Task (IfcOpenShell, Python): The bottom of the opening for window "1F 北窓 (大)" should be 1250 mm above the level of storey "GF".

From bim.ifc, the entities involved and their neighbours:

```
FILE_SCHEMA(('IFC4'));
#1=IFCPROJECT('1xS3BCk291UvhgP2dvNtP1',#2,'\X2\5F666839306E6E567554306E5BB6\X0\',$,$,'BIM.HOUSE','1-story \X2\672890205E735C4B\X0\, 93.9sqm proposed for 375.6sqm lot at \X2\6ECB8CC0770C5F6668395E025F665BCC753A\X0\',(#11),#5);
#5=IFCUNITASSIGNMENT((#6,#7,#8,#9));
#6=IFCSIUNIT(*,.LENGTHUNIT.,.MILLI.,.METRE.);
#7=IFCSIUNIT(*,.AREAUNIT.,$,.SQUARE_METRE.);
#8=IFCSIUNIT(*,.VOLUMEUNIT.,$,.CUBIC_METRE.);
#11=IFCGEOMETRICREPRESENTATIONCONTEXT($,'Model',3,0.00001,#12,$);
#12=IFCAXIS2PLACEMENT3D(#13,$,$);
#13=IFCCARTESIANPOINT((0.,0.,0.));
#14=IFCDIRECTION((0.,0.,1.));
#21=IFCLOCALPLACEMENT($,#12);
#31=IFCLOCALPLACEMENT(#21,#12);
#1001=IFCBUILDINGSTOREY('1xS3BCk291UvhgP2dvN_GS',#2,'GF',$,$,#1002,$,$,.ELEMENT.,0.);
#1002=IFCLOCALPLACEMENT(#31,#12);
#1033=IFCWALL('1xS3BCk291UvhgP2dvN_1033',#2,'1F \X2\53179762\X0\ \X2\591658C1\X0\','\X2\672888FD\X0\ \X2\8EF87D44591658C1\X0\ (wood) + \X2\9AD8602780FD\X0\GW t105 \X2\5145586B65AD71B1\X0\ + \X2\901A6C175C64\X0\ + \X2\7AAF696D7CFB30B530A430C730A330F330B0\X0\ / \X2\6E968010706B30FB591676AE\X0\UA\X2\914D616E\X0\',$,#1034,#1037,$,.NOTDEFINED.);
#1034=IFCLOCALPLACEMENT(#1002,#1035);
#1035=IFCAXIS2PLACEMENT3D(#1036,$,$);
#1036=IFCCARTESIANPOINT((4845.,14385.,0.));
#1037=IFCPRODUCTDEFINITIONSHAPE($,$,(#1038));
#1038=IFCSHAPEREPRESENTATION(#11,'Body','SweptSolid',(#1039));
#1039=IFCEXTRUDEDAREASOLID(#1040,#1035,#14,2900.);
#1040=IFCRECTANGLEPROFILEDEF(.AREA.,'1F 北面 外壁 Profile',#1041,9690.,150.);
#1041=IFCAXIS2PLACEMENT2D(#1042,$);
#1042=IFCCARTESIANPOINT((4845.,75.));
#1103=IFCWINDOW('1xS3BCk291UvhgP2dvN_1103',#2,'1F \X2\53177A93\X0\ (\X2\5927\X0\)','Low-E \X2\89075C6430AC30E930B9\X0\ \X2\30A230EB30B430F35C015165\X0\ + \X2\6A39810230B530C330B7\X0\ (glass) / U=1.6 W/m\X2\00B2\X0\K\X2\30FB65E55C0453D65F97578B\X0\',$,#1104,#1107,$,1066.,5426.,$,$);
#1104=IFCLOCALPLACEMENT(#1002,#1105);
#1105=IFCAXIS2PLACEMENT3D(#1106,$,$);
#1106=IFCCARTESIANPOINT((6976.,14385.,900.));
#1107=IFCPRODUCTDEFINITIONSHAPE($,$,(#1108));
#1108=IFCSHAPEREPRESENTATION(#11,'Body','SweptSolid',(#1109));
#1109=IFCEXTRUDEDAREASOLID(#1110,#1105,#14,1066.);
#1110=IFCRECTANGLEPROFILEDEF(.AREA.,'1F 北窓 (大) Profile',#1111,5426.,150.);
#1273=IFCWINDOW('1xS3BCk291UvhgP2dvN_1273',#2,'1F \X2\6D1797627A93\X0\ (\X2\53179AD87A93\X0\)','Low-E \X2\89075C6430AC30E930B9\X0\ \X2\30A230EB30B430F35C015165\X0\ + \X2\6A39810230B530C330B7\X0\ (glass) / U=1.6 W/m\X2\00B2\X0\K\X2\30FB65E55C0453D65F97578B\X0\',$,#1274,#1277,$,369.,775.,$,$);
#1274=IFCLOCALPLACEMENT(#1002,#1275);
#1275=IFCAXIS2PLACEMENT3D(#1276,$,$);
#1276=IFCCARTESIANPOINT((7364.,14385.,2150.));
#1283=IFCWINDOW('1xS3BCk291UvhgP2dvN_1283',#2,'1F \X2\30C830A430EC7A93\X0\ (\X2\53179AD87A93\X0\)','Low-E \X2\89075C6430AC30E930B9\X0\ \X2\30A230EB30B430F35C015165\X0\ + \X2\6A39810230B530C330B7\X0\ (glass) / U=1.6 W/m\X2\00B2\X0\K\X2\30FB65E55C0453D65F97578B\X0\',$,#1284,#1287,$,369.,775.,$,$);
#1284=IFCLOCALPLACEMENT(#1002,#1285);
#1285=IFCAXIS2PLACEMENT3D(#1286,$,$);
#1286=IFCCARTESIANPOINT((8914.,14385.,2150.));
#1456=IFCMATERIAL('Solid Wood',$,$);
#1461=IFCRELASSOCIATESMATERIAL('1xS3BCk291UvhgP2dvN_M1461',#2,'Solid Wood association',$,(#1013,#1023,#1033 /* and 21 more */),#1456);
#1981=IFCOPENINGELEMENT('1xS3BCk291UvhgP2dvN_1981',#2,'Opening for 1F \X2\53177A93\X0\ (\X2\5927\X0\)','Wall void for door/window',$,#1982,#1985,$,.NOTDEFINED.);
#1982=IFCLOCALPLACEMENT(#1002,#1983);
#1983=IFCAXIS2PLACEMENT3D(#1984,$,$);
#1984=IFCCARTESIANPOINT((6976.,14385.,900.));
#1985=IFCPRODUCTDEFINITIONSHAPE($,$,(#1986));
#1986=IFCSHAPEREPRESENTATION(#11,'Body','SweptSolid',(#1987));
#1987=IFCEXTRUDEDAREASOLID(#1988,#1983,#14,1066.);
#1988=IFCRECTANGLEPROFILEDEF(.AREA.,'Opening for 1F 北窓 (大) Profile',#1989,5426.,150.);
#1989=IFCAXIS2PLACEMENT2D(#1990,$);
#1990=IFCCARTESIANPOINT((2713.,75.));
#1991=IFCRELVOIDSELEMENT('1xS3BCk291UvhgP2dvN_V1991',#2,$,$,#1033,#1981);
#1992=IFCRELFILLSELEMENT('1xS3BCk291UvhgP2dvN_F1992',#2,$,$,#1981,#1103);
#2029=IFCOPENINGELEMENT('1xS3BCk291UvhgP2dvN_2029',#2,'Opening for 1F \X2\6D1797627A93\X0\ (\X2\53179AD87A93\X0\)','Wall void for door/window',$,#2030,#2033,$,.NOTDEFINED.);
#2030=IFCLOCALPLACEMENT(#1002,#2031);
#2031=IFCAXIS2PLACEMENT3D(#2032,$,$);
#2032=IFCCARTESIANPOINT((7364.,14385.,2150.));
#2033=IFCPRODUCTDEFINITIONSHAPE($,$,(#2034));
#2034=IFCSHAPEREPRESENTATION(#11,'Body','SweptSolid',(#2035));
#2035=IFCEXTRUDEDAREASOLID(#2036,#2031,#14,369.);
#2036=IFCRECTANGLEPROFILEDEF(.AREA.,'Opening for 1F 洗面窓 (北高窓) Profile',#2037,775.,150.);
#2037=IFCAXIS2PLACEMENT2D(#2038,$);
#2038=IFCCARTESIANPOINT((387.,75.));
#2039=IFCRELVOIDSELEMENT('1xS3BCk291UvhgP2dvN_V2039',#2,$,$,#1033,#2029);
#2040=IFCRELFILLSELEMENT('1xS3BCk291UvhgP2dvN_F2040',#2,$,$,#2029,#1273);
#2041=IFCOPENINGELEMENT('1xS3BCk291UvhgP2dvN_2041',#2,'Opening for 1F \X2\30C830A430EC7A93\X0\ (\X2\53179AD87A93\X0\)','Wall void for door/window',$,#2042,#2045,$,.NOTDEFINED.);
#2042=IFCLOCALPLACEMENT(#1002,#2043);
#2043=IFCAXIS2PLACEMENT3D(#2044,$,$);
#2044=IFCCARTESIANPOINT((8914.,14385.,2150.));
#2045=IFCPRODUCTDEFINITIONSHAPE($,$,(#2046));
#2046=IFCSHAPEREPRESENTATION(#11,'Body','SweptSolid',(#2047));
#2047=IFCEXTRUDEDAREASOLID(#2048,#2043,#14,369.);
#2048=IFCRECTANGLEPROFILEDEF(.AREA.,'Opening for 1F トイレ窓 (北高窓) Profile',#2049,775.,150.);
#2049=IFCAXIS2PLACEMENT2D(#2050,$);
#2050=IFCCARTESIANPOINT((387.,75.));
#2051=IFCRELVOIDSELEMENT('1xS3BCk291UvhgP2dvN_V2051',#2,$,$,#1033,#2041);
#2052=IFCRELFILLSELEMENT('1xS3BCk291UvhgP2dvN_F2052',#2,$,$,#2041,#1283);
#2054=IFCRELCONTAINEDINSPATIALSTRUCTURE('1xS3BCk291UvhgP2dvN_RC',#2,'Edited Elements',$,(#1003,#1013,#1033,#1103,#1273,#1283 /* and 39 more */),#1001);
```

```python
import numpy as np
import ifcopenshell
import ifcopenshell.api.geometry
import ifcopenshell.geom
import ifcopenshell.util.element
import ifcopenshell.util.placement
import ifcopenshell.util.shape
import ifcopenshell.util.unit

model = ifcopenshell.open("bim.ifc")
unit_scale = ifcopenshell.util.unit.calculate_unit_scale(model)

window = model.by_id(1103)
opening = window.FillsVoids[0].RelatingOpeningElement
storey = ifcopenshell.util.element.get_container(window, ifc_class="IfcBuildingStorey")
level = ifcopenshell.util.placement.get_local_placement(storey.ObjectPlacement)[2, 3]

# The opening's origin need not be at the sill, so measure its lowest point.
shape = ifcopenshell.geom.create_shape(ifcopenshell.geom.settings(), opening)
bottom = ifcopenshell.util.shape.get_shape_bottom_elevation(shape, shape.geometry) / unit_scale
dz = level + 1.25 / unit_scale - bottom

shift = np.array([0.0, 0.0, dz])
# The window is not placed relative to its opening, so move both.
for product in (opening, window):
    matrix = ifcopenshell.util.placement.get_local_placement(product.ObjectPlacement)
    matrix[:3, 3] += shift
    ifcopenshell.api.geometry.edit_object_placement(model, product=product, matrix=matrix, is_si=False)

print(f"moved by {dz * unit_scale:+.3f} m")

model.write("bim-out.ifc")
```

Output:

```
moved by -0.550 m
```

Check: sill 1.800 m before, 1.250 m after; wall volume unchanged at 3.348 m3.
